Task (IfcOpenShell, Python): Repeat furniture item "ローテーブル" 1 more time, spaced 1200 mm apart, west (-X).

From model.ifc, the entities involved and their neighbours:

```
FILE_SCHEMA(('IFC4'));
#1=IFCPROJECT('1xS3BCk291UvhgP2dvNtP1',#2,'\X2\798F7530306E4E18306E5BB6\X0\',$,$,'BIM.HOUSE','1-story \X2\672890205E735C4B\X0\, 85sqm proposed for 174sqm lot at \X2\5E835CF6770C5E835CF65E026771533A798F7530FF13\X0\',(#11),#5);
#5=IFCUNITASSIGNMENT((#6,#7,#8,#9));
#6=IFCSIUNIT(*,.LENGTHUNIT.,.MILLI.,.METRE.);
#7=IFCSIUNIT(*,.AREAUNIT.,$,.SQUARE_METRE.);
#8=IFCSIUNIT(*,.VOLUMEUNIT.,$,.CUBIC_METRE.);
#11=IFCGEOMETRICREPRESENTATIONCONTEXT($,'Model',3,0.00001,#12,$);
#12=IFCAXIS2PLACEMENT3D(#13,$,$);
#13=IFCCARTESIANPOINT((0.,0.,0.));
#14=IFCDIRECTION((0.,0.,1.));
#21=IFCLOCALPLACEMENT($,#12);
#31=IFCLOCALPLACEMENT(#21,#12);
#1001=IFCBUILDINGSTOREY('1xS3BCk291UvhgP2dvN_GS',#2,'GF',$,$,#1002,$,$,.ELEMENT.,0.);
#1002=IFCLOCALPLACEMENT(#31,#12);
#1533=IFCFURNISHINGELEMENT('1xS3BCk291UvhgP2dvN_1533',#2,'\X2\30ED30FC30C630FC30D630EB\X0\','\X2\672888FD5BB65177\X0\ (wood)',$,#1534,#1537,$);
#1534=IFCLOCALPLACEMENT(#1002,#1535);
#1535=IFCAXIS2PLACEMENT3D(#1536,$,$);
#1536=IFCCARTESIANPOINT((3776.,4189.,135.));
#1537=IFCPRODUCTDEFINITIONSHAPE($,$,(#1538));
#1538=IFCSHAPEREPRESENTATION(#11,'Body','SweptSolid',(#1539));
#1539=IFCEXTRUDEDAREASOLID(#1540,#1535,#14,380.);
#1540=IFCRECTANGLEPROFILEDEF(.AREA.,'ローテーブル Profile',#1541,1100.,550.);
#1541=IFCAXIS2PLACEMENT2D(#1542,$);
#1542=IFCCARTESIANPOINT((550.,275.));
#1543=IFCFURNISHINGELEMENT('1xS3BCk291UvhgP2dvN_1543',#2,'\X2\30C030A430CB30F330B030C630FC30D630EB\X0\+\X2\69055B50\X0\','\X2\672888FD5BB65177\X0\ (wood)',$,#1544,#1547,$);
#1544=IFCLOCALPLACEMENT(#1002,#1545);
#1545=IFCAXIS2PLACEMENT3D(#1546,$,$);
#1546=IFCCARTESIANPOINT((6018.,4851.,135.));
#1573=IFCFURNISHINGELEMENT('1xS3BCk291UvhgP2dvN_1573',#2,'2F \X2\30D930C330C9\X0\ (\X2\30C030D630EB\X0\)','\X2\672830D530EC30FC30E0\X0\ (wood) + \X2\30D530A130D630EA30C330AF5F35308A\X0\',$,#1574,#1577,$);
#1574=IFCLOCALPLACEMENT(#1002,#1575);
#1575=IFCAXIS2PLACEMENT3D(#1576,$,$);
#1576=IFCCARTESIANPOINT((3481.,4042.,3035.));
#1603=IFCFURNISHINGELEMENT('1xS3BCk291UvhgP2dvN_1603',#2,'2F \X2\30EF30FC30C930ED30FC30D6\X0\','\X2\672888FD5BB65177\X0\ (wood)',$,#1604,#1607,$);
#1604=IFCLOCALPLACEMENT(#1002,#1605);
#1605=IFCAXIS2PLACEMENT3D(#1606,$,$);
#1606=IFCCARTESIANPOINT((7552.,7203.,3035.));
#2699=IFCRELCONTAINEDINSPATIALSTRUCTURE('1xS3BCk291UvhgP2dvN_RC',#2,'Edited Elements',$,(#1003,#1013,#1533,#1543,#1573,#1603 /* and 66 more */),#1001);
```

```python
import numpy as np
import ifcopenshell
import ifcopenshell.api.geometry
import ifcopenshell.api.root
import ifcopenshell.util.element
import ifcopenshell.util.placement
import ifcopenshell.util.unit

model = ifcopenshell.open("model.ifc")
unit_scale = ifcopenshell.util.unit.calculate_unit_scale(model)


def reuse_history(source, copy):
    """copy_class also copies each property set's owner history, people and application; keep the originals."""
    for rel in copy.IsDefinedBy:
        if rel.is_a("IfcRelDefinesByProperties") and (history := rel.RelatingPropertyDefinition.OwnerHistory):
            rel.RelatingPropertyDefinition.OwnerHistory = source.OwnerHistory
            ifcopenshell.util.element.remove_deep2(model, history)


source = model.by_guid("1xS3BCk291UvhgP2dvN_1533")
base = ifcopenshell.util.placement.get_local_placement(source.ObjectPlacement)
step = np.array([-1.0, 0.0, 0.0]) * 1.2 / unit_scale

for i in range(1, 2):
    copy = ifcopenshell.api.root.copy_class(model, product=source)
    copy.Representation = ifcopenshell.util.element.copy_deep(
        model, source.Representation, exclude=["IfcGeometricRepresentationContext", "IfcRepresentationMap"]
    )
    reuse_history(source, copy)
    matrix = base.copy()
    matrix[:3, 3] += i * step
    print("added at", matrix[:3, 3].round(3) + 0.0)
    ifcopenshell.api.geometry.edit_object_placement(model, product=copy, matrix=matrix, is_si=False)

model.write("model-out.ifc")
```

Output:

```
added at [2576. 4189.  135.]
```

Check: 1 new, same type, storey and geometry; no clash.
